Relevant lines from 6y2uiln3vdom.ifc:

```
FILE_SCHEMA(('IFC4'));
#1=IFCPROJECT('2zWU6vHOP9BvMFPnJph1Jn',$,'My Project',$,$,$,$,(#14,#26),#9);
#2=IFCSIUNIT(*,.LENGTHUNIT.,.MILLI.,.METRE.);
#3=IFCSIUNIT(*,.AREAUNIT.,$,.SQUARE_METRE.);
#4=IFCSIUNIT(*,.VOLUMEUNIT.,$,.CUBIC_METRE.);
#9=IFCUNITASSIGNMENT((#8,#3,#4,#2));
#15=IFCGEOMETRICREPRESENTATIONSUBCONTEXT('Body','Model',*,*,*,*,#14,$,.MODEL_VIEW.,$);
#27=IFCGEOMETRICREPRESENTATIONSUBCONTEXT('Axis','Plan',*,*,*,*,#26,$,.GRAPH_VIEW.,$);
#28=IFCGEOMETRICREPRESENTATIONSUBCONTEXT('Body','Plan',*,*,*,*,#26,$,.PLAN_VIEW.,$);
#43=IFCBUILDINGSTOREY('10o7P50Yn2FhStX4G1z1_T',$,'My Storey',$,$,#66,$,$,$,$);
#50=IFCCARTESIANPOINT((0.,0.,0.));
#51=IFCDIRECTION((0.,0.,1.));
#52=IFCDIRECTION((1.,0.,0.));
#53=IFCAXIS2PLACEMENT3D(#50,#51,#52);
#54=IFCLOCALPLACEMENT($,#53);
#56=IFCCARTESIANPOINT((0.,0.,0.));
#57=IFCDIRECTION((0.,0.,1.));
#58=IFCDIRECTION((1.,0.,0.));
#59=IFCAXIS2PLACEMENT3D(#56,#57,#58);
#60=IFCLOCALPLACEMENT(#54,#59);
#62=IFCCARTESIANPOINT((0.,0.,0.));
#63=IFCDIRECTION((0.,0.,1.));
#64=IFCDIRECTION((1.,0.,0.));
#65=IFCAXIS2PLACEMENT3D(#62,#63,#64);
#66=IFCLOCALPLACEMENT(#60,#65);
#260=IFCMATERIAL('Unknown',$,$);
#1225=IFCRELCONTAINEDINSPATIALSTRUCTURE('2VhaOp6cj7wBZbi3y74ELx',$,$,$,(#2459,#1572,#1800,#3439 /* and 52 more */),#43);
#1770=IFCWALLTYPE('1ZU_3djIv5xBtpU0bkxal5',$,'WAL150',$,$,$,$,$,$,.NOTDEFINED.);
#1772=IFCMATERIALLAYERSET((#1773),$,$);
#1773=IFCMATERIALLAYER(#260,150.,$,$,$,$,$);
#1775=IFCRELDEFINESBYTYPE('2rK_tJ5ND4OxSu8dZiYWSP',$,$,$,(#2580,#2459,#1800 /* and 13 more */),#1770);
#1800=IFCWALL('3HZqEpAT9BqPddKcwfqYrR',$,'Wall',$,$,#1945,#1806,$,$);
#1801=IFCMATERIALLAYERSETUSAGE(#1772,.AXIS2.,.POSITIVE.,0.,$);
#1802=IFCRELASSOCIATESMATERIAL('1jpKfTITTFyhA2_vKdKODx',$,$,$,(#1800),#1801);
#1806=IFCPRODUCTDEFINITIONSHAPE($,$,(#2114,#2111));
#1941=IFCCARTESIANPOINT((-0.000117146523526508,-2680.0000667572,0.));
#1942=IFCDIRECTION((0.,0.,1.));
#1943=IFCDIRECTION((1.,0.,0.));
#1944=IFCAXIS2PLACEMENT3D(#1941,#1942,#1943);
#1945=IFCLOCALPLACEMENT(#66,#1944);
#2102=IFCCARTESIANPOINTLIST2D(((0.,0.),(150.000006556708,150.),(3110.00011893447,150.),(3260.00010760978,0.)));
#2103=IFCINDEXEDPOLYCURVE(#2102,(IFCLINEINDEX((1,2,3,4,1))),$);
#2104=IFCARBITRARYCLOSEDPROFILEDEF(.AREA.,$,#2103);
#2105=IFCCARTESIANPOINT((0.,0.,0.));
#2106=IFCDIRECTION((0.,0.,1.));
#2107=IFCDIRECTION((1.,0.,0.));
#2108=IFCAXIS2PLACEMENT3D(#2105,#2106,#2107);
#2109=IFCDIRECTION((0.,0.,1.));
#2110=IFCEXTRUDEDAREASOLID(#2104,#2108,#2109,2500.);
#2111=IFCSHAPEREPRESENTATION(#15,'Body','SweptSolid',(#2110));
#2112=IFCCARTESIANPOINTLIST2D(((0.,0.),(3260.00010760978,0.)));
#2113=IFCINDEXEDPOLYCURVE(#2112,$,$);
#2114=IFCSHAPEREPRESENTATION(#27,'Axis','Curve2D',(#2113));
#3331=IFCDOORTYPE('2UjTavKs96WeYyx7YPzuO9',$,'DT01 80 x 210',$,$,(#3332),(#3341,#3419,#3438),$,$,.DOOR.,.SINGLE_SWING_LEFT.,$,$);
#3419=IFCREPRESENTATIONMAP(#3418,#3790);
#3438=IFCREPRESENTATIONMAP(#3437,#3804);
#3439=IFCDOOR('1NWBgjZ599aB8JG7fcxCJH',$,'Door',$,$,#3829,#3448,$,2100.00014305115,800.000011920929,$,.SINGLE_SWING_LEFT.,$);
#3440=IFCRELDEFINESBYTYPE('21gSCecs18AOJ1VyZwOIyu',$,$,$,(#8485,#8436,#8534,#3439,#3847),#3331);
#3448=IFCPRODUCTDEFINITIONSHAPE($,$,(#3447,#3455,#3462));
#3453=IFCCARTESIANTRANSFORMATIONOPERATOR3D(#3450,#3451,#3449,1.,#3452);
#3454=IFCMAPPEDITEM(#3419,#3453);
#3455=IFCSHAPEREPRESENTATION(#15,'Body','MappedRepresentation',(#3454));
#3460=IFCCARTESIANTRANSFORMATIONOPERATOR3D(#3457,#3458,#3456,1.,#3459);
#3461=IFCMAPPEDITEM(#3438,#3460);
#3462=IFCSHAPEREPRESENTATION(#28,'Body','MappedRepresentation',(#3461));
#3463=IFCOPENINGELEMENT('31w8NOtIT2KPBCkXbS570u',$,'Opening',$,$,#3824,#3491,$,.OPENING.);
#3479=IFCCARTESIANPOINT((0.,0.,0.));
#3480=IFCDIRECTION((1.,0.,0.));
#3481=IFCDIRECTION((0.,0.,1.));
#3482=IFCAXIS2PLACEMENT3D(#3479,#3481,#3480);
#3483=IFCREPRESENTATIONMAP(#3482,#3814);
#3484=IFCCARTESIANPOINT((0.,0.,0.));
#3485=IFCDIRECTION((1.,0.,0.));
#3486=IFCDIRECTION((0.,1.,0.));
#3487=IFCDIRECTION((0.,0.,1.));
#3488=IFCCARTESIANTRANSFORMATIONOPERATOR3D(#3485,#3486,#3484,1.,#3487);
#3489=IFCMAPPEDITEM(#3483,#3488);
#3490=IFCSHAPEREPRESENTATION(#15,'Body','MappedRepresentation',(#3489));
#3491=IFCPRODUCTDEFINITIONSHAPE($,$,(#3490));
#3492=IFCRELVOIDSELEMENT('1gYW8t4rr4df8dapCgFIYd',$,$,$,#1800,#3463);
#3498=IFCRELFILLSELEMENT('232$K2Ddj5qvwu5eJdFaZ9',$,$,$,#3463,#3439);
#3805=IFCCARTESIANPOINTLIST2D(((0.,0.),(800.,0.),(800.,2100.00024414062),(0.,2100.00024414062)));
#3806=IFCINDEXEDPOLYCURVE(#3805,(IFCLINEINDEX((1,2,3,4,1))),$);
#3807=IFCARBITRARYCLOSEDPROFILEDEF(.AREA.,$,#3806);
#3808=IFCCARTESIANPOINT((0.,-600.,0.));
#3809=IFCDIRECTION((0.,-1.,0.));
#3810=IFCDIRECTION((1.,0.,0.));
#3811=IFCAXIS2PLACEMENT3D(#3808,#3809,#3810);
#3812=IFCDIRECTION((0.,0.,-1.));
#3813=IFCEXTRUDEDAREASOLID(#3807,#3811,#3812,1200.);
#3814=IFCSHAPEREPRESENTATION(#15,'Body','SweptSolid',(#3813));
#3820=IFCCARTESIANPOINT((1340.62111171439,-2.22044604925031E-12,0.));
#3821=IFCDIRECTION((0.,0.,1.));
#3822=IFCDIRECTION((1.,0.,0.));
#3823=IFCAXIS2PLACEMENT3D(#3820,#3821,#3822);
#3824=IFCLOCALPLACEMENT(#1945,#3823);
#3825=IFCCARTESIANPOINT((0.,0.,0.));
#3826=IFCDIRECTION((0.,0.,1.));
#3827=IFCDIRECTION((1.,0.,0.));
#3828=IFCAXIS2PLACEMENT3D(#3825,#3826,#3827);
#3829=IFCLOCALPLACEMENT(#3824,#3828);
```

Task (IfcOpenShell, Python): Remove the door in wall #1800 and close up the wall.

```python
import ifcopenshell
import ifcopenshell.api.feature
import ifcopenshell.api.root
import ifcopenshell.geom
import ifcopenshell.util.shape

model = ifcopenshell.open("6y2uiln3vdom.ifc")
settings = ifcopenshell.geom.settings()


def volume(element):
    """Net volume in cubic metres, openings subtracted."""
    shape = ifcopenshell.geom.create_shape(settings, element)
    return ifcopenshell.util.shape.get_volume(shape.geometry)


door = model.by_id(3439)
opening = door.FillsVoids[0].RelatingOpeningElement
wall = opening.VoidsElements[0].RelatingBuildingElement
before = volume(wall)

ifcopenshell.api.root.remove_product(model, product=door)
ifcopenshell.api.feature.remove_feature(model, feature=opening)

after = volume(wall)

print(f"wall volume {before:.3f} -> {after:.3f} m3")

model.write("6y2uiln3vdom-out.ifc")
```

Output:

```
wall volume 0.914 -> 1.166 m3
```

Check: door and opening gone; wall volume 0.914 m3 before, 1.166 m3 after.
